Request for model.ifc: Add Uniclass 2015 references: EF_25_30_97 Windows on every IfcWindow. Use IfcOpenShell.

First a look at what the model holds.

```python
import ifcopenshell

model = ifcopenshell.open("model.ifc")
print(model.schema)
print("classifications:", [c.Name for c in model.by_type("IfcClassification")])
for ifc_class in ("IfcDoor", "IfcRoof", "IfcStair", "IfcWall", "IfcWindow"):
    print(ifc_class, len(model.by_type(ifc_class)))
```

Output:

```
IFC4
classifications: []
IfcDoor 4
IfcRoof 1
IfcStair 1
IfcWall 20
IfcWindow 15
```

```python
import ifcopenshell
import ifcopenshell.api.classification

model = ifcopenshell.open("model.ifc")

system = ifcopenshell.api.classification.add_classification(model, classification="Uniclass 2015")

codes = {
    "IfcWindow": ("EF_25_30_97", "Windows"),
}
for ifc_class, (code, name) in codes.items():
    products = model.by_type(ifc_class)
    ifcopenshell.api.classification.add_reference(
        model, products=products, classification=system, identification=code, name=name
    )
    print(code, len(products))

model.write("model-out.ifc")
```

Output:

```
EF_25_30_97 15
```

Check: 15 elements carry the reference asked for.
